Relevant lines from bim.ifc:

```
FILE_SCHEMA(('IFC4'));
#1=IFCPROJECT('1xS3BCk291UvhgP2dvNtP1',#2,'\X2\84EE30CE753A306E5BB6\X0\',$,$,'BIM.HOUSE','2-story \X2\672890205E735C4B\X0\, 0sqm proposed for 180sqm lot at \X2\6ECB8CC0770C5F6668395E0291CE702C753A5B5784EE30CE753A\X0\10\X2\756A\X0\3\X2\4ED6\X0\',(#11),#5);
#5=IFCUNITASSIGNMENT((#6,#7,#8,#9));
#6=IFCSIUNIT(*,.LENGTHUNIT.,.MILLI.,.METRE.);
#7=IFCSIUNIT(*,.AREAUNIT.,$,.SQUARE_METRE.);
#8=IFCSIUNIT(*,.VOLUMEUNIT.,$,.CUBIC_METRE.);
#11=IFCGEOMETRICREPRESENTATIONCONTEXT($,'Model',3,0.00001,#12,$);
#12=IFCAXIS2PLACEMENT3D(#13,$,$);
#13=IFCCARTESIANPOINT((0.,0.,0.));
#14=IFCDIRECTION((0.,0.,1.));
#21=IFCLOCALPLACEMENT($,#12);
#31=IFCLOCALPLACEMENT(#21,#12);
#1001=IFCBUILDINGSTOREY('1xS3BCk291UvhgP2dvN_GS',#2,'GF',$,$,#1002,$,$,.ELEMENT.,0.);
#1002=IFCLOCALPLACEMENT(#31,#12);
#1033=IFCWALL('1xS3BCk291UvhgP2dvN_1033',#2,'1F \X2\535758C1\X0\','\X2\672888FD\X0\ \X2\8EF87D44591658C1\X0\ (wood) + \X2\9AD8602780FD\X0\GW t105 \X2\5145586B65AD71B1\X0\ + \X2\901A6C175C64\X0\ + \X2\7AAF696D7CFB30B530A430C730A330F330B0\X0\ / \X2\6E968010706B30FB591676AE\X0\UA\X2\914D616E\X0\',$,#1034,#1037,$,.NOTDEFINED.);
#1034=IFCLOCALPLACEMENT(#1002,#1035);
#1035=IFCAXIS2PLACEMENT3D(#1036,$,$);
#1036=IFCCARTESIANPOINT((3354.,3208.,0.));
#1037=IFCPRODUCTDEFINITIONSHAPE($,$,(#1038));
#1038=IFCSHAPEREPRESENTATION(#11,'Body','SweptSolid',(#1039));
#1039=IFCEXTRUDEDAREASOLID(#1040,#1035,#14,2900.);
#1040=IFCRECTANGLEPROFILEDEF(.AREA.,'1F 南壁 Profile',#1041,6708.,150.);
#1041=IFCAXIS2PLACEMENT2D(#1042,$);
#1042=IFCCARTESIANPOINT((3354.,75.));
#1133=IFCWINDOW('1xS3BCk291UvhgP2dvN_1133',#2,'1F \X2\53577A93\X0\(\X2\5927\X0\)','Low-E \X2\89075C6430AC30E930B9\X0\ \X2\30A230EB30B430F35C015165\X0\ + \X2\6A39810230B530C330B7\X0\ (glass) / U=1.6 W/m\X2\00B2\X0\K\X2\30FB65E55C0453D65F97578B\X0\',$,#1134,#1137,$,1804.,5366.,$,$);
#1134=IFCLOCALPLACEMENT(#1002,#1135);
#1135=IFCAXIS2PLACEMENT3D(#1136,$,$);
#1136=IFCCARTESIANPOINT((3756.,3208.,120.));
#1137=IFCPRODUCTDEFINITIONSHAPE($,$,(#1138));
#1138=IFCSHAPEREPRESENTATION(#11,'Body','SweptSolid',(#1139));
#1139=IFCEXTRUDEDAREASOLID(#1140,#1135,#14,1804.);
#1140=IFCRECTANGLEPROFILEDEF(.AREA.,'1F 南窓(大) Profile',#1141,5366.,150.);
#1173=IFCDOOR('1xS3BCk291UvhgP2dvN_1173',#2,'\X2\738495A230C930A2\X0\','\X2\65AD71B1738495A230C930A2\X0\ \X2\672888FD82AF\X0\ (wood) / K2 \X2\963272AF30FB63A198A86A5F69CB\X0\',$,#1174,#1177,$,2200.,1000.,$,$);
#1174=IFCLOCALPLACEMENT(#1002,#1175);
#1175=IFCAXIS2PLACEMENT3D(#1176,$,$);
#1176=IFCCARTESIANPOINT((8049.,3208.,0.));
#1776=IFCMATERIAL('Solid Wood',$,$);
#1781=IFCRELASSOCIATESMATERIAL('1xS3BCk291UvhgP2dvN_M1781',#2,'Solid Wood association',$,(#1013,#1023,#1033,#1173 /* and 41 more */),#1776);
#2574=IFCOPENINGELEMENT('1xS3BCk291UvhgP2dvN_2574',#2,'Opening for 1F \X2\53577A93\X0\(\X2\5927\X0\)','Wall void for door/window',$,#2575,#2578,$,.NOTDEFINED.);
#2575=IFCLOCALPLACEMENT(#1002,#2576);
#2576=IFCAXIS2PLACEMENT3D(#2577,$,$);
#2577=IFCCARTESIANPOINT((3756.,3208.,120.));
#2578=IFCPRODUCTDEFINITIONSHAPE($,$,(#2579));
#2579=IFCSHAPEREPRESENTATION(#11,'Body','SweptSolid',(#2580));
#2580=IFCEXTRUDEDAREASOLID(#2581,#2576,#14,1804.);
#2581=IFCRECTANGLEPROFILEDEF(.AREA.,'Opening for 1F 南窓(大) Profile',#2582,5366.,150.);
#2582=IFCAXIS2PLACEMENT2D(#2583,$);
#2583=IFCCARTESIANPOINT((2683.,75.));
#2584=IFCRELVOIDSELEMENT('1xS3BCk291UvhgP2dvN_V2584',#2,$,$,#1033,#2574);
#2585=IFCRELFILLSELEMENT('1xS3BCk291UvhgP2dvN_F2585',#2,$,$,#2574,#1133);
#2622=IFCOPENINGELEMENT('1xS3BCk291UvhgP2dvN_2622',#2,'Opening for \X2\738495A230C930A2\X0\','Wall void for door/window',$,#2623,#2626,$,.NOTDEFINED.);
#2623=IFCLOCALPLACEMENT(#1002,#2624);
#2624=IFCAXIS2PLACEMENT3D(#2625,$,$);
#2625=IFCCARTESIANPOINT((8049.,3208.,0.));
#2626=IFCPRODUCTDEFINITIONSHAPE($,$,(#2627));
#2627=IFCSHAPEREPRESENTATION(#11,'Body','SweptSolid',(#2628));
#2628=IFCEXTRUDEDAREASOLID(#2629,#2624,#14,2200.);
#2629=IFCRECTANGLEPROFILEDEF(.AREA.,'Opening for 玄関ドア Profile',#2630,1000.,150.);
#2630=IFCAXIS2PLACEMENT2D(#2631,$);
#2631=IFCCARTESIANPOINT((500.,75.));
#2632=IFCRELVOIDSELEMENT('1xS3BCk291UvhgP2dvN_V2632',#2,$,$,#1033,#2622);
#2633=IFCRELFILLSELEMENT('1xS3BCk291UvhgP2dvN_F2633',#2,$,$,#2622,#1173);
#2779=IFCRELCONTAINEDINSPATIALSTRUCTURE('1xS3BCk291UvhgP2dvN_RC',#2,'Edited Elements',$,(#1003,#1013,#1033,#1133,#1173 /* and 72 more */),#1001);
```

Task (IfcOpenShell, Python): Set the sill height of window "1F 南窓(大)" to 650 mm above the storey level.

```python
import numpy as np
import ifcopenshell
import ifcopenshell.api.geometry
import ifcopenshell.geom
import ifcopenshell.util.element
import ifcopenshell.util.placement
import ifcopenshell.util.shape
import ifcopenshell.util.unit

model = ifcopenshell.open("bim.ifc")
unit_scale = ifcopenshell.util.unit.calculate_unit_scale(model)

window = model.by_guid("1xS3BCk291UvhgP2dvN_1133")
opening = window.FillsVoids[0].RelatingOpeningElement
storey = ifcopenshell.util.element.get_container(window, ifc_class="IfcBuildingStorey")
level = ifcopenshell.util.placement.get_local_placement(storey.ObjectPlacement)[2, 3]

# The opening's origin need not be at the sill, so measure its lowest point.
shape = ifcopenshell.geom.create_shape(ifcopenshell.geom.settings(), opening)
bottom = ifcopenshell.util.shape.get_shape_bottom_elevation(shape, shape.geometry) / unit_scale
dz = level + 0.65 / unit_scale - bottom

shift = np.array([0.0, 0.0, dz])
# The window is not placed relative to its opening, so move both.
for product in (opening, window):
    matrix = ifcopenshell.util.placement.get_local_placement(product.ObjectPlacement)
    matrix[:3, 3] += shift
    ifcopenshell.api.geometry.edit_object_placement(model, product=product, matrix=matrix, is_si=False)

print(f"moved by {dz * unit_scale:+.3f} m")

model.write("bim_v2.ifc")
```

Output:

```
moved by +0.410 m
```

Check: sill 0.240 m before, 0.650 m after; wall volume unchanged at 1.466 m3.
